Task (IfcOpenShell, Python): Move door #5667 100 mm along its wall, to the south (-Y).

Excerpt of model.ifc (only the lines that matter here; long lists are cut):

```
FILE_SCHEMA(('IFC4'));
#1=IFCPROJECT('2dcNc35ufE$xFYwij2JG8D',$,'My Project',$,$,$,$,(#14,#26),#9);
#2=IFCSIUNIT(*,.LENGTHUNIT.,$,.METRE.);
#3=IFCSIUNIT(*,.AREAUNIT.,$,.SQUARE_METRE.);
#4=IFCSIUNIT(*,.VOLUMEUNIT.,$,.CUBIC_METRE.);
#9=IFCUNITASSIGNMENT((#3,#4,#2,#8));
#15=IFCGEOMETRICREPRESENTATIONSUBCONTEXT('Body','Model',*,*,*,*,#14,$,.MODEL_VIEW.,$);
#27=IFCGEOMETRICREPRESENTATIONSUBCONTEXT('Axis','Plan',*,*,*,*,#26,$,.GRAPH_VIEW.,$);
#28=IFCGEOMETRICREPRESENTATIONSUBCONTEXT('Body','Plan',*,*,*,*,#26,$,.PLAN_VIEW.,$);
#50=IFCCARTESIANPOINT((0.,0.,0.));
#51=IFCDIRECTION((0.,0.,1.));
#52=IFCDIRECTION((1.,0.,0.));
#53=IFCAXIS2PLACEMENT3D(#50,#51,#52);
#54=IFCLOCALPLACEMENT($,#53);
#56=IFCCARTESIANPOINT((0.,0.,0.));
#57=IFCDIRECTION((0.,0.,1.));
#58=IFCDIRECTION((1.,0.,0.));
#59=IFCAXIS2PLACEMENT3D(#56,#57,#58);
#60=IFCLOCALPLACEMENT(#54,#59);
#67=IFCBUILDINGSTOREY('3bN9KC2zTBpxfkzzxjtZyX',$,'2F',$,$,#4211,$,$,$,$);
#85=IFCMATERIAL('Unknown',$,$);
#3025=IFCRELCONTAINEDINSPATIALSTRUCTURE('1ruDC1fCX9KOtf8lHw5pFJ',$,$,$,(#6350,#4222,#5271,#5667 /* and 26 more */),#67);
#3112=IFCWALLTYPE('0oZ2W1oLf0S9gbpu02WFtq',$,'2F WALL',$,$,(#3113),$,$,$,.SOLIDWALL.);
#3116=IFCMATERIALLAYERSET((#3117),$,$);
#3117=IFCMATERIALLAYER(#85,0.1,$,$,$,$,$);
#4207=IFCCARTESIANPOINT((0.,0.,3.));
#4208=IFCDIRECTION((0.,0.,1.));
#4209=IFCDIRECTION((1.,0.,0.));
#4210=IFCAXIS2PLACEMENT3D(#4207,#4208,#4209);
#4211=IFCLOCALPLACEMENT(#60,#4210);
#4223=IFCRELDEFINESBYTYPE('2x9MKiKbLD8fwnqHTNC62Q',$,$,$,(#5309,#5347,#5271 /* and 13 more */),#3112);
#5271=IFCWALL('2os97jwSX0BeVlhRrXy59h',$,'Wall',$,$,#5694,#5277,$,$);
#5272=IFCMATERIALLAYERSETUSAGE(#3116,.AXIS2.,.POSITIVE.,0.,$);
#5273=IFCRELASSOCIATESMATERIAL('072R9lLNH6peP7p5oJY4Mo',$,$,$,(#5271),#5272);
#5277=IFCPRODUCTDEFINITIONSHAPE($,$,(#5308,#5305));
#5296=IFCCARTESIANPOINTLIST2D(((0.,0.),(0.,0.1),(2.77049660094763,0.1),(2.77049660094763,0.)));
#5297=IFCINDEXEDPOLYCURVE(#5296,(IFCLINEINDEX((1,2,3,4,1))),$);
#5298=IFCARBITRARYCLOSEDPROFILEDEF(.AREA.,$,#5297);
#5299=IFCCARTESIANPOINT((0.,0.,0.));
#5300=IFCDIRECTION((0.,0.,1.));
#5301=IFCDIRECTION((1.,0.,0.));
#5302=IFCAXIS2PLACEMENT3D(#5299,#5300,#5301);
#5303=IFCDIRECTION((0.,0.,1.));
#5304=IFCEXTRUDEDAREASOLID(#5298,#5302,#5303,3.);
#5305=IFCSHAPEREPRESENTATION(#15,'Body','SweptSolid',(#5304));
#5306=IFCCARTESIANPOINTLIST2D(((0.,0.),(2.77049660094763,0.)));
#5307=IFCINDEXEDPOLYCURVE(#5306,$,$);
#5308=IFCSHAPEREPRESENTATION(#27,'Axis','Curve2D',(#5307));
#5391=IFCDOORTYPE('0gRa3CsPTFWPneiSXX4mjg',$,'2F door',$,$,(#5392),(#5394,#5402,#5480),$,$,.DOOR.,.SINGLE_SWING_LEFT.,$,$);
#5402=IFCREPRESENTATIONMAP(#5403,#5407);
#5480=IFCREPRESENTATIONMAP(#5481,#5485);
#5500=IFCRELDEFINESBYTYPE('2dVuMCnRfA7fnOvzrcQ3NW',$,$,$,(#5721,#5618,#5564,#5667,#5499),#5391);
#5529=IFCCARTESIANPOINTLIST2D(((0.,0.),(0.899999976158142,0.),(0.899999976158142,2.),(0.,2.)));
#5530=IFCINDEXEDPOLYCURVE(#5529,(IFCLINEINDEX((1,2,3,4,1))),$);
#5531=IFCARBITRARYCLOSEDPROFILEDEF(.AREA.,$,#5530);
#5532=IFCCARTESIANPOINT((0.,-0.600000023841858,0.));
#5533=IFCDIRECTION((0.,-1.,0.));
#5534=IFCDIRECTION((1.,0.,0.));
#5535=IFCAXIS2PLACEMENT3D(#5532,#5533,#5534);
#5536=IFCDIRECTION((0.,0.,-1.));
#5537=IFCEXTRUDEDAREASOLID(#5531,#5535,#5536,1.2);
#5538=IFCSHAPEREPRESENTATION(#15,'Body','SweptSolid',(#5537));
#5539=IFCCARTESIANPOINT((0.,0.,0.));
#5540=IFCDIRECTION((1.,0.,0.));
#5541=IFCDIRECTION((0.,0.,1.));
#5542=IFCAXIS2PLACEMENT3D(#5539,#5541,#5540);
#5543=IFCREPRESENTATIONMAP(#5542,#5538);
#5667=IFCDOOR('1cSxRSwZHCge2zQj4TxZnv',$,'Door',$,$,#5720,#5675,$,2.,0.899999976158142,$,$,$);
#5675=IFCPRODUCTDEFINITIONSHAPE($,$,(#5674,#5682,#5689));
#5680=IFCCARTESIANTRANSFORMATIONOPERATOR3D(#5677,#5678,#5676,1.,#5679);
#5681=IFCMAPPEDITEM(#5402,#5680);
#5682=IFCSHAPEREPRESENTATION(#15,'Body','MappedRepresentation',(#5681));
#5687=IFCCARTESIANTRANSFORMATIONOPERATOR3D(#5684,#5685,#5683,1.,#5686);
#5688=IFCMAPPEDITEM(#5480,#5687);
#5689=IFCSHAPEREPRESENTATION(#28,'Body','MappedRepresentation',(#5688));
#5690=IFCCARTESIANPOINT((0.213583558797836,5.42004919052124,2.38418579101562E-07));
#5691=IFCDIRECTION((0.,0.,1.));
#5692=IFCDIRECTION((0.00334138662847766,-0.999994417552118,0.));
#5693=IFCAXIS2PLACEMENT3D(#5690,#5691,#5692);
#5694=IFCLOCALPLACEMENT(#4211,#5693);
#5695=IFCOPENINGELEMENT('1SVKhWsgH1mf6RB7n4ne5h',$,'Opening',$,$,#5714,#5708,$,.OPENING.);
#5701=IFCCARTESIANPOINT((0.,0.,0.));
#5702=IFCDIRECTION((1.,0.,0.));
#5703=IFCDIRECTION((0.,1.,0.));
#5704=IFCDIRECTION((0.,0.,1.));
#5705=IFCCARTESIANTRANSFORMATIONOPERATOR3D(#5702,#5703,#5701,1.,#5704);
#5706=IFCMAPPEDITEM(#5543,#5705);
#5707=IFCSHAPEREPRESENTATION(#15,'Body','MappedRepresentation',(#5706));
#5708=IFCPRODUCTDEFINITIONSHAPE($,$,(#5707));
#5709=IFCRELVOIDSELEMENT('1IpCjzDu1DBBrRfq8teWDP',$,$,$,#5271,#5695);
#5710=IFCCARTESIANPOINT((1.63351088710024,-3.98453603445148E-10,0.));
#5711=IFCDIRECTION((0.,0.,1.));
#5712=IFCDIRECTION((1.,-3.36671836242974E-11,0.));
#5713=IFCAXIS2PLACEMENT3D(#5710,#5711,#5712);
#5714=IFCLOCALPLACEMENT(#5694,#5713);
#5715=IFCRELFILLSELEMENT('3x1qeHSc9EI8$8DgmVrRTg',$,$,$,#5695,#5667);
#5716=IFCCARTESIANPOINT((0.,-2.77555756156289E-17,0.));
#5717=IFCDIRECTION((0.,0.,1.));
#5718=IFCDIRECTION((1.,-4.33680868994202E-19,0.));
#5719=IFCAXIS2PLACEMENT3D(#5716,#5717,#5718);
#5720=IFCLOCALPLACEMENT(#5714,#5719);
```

```python
import ifcopenshell
import ifcopenshell.api.geometry
import ifcopenshell.util.placement

model = ifcopenshell.open("model.ifc")

door = model.by_id(5667)
opening = door.FillsVoids[0].RelatingOpeningElement
wall = opening.VoidsElements[0].RelatingBuildingElement

wall_matrix = ifcopenshell.util.placement.get_local_placement(wall.ObjectPlacement)
shift = wall_matrix[:3, 0] * 0.1
before = ifcopenshell.util.placement.get_local_placement(door.ObjectPlacement)[:3, 3].copy()

# The door is placed relative to its opening, so it follows when the opening moves.
matrix = ifcopenshell.util.placement.get_local_placement(opening.ObjectPlacement)
matrix[:3, 3] += shift
ifcopenshell.api.geometry.edit_object_placement(
    model, product=opening, matrix=matrix, is_si=False, should_transform_children=True
)

after = ifcopenshell.util.placement.get_local_placement(door.ObjectPlacement)[:3, 3]
print("door moved by", (after - before).round(3) + 0.0)

model.write("model_updated.ifc")
```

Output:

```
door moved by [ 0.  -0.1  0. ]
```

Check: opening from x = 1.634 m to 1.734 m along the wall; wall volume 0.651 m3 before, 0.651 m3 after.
